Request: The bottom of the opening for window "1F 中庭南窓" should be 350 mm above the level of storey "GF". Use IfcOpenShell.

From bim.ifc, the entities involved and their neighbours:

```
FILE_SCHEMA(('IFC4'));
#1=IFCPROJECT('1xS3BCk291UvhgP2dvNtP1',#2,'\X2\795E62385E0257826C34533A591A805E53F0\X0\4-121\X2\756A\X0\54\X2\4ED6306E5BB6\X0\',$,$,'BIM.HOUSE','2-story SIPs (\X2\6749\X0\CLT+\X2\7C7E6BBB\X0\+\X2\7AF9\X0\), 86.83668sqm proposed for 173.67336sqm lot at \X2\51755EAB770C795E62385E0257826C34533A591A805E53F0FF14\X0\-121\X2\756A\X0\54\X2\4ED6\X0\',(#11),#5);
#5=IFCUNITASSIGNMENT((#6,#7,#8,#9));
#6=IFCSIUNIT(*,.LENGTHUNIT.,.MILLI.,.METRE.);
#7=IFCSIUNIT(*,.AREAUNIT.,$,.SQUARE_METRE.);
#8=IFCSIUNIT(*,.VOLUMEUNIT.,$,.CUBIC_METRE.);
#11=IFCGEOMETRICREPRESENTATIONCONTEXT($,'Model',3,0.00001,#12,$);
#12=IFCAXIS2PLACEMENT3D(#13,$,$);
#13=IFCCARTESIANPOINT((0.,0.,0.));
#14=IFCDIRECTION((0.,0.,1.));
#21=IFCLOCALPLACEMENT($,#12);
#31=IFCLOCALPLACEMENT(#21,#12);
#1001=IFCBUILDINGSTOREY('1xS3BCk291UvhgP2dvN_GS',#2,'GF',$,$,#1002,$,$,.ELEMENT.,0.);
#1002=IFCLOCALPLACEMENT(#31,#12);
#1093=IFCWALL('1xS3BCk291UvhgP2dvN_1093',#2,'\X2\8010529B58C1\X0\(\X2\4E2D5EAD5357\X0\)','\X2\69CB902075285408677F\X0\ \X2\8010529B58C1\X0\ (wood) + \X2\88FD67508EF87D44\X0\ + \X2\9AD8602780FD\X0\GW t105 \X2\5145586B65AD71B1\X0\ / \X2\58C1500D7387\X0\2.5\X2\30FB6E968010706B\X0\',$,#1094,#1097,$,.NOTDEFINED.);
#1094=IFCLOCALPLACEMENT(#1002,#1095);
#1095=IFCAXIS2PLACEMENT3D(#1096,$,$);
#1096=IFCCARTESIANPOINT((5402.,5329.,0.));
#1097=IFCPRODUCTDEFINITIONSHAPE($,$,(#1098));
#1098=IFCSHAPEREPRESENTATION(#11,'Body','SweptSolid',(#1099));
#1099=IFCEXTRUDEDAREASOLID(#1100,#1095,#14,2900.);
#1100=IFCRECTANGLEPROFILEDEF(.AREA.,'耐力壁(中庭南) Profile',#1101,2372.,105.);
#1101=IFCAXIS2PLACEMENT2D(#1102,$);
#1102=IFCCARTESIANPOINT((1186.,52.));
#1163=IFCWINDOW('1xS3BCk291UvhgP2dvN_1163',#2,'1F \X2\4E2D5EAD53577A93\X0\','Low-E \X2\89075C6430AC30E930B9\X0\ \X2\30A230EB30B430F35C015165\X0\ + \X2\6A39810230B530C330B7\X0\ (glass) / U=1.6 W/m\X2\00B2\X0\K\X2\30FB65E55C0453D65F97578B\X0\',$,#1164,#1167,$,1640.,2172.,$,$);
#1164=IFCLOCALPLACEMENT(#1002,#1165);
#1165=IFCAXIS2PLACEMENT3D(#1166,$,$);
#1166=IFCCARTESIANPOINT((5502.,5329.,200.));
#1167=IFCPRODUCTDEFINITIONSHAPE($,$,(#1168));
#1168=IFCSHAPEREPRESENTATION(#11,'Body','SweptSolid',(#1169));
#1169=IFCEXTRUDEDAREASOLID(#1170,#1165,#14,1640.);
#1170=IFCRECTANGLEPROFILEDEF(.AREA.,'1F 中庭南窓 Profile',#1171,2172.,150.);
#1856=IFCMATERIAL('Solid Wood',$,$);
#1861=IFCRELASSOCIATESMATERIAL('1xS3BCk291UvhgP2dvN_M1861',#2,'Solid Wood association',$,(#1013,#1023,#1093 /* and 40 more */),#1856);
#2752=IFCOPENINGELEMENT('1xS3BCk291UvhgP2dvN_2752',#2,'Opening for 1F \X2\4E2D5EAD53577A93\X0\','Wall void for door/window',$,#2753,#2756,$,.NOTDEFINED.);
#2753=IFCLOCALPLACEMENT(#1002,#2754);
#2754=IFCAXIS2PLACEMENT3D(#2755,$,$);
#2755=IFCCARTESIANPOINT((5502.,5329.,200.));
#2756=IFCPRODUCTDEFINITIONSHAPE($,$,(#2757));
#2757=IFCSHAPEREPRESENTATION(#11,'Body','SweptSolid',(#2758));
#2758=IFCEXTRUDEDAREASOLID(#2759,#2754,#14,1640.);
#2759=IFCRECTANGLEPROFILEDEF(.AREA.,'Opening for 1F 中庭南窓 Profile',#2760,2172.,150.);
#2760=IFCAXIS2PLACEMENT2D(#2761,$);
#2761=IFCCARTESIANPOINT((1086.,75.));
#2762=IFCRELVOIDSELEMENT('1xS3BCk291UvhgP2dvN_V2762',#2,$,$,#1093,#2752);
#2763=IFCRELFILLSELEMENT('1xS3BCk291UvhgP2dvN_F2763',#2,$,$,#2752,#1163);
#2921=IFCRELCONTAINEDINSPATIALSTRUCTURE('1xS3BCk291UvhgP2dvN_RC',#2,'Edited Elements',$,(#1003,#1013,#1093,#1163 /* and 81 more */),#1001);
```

```python
import numpy as np
import ifcopenshell
import ifcopenshell.api.geometry
import ifcopenshell.geom
import ifcopenshell.util.element
import ifcopenshell.util.placement
import ifcopenshell.util.shape
import ifcopenshell.util.unit

model = ifcopenshell.open("bim.ifc")
unit_scale = ifcopenshell.util.unit.calculate_unit_scale(model)

window = model.by_guid("1xS3BCk291UvhgP2dvN_1163")
opening = window.FillsVoids[0].RelatingOpeningElement
storey = ifcopenshell.util.element.get_container(window, ifc_class="IfcBuildingStorey")
level = ifcopenshell.util.placement.get_local_placement(storey.ObjectPlacement)[2, 3]

# The opening's origin need not be at the sill, so measure its lowest point.
shape = ifcopenshell.geom.create_shape(ifcopenshell.geom.settings(), opening)
bottom = ifcopenshell.util.shape.get_shape_bottom_elevation(shape, shape.geometry) / unit_scale
dz = level + 350.0 - bottom

shift = np.array([0.0, 0.0, dz])
# The window is not placed relative to its opening, so move both.
for product in (opening, window):
    matrix = ifcopenshell.util.placement.get_local_placement(product.ObjectPlacement)
    matrix[:3, 3] += shift
    ifcopenshell.api.geometry.edit_object_placement(model, product=product, matrix=matrix, is_si=False)

print(f"moved by {dz * unit_scale:+.3f} m")

model.write("bim_v2.ifc")
```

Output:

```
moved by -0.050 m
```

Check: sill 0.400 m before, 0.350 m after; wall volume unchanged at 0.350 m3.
